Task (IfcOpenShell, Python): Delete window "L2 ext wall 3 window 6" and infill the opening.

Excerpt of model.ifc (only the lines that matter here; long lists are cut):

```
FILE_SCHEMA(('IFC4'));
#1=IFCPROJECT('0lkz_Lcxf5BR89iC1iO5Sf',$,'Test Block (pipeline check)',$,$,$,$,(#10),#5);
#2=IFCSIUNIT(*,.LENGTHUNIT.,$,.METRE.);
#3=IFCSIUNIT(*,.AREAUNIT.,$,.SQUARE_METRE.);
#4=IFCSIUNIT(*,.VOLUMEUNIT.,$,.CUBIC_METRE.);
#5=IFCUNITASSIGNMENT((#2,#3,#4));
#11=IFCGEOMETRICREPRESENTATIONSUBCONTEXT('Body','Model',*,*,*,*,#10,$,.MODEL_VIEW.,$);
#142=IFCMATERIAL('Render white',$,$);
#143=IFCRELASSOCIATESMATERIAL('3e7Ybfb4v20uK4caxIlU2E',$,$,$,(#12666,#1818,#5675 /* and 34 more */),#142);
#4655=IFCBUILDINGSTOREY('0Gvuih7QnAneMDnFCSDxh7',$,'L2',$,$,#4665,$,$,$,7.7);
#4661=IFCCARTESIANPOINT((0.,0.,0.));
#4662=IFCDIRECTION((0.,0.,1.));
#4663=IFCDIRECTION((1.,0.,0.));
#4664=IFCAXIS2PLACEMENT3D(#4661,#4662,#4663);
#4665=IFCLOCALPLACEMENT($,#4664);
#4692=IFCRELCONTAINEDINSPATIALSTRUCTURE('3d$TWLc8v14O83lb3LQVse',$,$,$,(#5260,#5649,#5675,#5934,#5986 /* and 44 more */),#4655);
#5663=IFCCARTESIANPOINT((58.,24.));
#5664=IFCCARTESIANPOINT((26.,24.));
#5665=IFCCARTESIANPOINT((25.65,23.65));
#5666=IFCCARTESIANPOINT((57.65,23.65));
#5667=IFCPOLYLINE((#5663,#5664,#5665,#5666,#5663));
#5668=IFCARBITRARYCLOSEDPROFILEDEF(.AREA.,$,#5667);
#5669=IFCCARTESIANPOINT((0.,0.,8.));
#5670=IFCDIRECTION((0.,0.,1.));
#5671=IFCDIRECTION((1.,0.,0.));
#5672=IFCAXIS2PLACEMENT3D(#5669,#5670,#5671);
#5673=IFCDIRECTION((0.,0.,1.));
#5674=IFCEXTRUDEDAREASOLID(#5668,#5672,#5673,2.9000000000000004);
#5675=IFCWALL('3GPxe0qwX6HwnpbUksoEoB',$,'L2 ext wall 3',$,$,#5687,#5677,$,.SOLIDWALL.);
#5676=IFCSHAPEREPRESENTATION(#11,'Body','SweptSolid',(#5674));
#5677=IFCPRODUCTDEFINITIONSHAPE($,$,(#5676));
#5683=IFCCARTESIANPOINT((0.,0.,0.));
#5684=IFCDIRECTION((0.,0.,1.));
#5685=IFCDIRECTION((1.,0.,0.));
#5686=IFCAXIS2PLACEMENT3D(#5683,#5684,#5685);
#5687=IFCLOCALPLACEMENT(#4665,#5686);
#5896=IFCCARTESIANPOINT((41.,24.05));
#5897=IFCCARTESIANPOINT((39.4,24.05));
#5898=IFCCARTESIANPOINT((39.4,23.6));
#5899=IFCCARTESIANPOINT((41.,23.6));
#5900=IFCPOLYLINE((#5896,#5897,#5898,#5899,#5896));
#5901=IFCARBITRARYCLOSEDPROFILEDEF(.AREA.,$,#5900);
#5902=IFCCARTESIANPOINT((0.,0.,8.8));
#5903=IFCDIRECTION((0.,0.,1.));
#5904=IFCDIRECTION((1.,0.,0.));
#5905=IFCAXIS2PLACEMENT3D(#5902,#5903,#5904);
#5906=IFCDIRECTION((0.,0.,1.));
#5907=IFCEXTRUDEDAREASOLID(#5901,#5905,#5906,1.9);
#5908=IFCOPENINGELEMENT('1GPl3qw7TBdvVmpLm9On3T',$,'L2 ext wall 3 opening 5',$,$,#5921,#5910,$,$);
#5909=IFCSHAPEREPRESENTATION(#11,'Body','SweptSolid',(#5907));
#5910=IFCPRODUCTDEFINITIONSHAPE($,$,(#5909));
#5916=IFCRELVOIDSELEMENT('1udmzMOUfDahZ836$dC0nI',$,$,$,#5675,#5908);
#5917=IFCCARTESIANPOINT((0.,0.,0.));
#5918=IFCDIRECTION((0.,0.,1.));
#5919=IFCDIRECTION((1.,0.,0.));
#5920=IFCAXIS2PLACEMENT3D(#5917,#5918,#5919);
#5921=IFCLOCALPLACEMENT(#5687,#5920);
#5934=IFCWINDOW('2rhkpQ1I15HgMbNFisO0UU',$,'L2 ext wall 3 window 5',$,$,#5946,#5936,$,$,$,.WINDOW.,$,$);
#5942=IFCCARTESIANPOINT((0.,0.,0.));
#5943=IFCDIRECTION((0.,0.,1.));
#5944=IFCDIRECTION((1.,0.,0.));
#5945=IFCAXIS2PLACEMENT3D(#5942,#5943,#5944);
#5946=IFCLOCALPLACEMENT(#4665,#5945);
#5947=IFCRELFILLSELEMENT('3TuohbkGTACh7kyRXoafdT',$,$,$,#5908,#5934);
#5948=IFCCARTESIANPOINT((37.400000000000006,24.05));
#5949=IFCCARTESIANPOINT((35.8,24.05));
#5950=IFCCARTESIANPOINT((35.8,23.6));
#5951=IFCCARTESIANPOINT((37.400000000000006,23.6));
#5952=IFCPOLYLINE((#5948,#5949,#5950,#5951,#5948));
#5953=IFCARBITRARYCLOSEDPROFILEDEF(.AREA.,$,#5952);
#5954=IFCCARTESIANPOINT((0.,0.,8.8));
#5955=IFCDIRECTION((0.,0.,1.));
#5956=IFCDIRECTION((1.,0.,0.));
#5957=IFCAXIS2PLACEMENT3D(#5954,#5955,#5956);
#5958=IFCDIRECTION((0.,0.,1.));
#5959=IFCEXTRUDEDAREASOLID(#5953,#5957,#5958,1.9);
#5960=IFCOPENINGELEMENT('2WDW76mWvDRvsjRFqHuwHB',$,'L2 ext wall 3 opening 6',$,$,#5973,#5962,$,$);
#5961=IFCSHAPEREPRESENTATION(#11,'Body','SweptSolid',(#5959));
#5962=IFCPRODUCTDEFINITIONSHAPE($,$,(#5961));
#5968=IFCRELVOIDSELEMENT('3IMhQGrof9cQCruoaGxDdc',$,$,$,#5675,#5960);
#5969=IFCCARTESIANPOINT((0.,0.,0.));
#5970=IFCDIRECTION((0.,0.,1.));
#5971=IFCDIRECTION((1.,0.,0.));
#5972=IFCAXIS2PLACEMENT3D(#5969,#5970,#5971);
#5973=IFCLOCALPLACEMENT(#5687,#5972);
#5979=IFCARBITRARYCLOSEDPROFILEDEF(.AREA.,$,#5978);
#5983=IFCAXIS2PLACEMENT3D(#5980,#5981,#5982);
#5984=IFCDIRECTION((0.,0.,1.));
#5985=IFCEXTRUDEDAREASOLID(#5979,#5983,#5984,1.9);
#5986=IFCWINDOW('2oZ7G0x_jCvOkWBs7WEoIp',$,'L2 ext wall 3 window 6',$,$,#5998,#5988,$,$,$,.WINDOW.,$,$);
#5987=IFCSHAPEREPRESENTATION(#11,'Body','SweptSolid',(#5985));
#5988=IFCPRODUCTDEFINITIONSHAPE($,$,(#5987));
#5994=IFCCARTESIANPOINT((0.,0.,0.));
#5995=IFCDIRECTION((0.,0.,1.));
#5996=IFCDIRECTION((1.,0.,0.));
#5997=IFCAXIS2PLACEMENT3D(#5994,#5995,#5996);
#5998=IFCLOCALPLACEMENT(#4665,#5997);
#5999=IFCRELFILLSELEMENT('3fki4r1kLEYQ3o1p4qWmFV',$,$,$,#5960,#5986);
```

```python
import ifcopenshell
import ifcopenshell.api.feature
import ifcopenshell.api.root
import ifcopenshell.geom
import ifcopenshell.util.shape

model = ifcopenshell.open("model.ifc")
settings = ifcopenshell.geom.settings()


def volume(element):
    """Net volume in cubic metres, openings subtracted."""
    shape = ifcopenshell.geom.create_shape(settings, element)
    return ifcopenshell.util.shape.get_volume(shape.geometry)


window = model.by_guid("2oZ7G0x_jCvOkWBs7WEoIp")
opening = window.FillsVoids[0].RelatingOpeningElement
wall = opening.VoidsElements[0].RelatingBuildingElement
before = volume(wall)

ifcopenshell.api.root.remove_product(model, product=window)
ifcopenshell.api.feature.remove_feature(model, feature=opening)

after = volume(wall)

print(f"wall volume {before:.3f} -> {after:.3f} m3")

model.write("model_edited.ifc")
```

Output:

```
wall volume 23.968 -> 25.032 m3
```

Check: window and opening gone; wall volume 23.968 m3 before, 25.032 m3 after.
